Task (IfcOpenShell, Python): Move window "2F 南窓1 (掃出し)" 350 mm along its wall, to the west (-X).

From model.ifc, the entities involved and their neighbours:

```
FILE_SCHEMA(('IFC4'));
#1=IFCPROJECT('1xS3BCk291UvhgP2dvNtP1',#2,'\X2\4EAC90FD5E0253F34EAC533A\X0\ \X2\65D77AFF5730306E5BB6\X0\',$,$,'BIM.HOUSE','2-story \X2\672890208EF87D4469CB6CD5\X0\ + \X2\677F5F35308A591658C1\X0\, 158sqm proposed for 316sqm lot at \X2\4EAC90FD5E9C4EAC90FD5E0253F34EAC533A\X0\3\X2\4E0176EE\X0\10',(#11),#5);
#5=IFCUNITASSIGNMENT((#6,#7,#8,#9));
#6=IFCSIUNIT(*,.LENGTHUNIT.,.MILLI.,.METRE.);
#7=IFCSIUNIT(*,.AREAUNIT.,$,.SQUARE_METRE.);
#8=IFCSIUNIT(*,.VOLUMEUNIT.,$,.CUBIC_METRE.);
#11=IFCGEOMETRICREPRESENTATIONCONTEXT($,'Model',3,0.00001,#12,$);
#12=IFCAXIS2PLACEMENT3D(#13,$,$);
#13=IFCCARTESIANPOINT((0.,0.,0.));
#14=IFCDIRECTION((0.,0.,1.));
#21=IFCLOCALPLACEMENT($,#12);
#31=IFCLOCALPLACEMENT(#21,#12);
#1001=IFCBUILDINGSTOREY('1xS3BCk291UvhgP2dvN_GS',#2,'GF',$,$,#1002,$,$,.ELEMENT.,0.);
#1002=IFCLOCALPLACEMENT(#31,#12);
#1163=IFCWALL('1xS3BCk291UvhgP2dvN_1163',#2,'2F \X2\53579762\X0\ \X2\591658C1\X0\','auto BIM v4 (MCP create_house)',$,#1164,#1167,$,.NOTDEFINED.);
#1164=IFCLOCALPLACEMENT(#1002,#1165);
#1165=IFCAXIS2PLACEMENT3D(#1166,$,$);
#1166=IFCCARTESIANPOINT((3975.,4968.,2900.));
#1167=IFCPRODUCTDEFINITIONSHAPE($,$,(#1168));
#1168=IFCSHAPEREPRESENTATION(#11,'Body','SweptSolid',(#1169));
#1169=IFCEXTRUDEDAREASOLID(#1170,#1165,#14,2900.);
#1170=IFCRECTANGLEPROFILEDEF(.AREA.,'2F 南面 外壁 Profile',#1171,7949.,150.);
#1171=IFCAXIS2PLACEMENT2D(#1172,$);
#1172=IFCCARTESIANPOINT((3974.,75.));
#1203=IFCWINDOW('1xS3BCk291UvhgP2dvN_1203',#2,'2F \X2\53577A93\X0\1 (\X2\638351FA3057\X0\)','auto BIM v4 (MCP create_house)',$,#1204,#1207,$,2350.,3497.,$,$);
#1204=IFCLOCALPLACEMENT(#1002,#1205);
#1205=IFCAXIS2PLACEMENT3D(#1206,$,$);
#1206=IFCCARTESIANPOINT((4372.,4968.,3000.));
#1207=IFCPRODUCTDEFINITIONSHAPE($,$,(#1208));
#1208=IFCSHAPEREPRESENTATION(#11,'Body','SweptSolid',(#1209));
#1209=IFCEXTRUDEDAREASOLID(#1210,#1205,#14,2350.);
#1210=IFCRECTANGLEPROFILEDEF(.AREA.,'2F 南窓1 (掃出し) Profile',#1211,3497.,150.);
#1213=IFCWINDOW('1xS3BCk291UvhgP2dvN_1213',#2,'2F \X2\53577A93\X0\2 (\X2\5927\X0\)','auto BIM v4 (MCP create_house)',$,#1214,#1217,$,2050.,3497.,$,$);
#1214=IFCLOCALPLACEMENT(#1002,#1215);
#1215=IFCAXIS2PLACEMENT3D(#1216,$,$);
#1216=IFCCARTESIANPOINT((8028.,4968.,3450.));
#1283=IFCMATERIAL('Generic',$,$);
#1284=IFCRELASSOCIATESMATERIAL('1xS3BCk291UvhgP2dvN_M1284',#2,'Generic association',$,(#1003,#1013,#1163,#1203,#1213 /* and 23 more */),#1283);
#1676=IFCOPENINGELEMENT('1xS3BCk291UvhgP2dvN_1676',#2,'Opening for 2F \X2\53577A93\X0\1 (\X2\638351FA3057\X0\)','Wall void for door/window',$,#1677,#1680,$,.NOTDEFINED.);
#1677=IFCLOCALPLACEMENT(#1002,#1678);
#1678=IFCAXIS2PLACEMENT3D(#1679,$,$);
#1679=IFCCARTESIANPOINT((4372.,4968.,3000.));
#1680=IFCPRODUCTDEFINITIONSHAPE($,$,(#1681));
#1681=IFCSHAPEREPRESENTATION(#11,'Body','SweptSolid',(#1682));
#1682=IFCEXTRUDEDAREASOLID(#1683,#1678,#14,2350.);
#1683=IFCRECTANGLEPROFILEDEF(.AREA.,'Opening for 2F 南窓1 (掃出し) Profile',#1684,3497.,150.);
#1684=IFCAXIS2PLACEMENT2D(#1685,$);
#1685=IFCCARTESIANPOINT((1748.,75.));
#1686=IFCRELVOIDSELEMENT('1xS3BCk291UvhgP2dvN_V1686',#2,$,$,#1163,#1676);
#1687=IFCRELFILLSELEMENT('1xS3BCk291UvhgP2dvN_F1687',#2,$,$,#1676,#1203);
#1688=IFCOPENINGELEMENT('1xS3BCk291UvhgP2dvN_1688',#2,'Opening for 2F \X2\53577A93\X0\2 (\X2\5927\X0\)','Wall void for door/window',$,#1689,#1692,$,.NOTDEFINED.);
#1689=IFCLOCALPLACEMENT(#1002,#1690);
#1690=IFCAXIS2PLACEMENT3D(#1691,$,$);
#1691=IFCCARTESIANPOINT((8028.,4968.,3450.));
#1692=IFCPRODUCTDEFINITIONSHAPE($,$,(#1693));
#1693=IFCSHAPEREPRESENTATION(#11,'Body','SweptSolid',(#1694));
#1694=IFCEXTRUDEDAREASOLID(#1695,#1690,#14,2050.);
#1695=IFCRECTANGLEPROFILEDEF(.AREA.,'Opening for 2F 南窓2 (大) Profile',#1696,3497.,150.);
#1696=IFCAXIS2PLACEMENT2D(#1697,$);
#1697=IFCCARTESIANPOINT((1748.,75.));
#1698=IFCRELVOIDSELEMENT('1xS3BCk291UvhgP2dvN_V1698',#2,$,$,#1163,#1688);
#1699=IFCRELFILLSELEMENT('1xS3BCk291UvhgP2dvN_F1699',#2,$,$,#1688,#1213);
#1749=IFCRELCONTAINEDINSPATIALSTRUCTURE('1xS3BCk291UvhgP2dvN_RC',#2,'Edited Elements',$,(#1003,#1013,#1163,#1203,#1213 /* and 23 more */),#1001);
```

```python
import ifcopenshell
import ifcopenshell.api.geometry
import ifcopenshell.util.placement

model = ifcopenshell.open("model.ifc")

window = model.by_id(1203)
opening = window.FillsVoids[0].RelatingOpeningElement
wall = opening.VoidsElements[0].RelatingBuildingElement

wall_matrix = ifcopenshell.util.placement.get_local_placement(wall.ObjectPlacement)
shift = wall_matrix[:3, 0] * -350.0
before = ifcopenshell.util.placement.get_local_placement(window.ObjectPlacement)[:3, 3].copy()

# The window is not placed relative to its opening, so move both.
for product in (opening, window):
    matrix = ifcopenshell.util.placement.get_local_placement(product.ObjectPlacement)
    matrix[:3, 3] += shift
    ifcopenshell.api.geometry.edit_object_placement(model, product=product, matrix=matrix, is_si=False)

after = ifcopenshell.util.placement.get_local_placement(window.ObjectPlacement)[:3, 3]
print("window moved by", (after - before).round(3) + 0.0)

model.write("model_rev.ifc")
```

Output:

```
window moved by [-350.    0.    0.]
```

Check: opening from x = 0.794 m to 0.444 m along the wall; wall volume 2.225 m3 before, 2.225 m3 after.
